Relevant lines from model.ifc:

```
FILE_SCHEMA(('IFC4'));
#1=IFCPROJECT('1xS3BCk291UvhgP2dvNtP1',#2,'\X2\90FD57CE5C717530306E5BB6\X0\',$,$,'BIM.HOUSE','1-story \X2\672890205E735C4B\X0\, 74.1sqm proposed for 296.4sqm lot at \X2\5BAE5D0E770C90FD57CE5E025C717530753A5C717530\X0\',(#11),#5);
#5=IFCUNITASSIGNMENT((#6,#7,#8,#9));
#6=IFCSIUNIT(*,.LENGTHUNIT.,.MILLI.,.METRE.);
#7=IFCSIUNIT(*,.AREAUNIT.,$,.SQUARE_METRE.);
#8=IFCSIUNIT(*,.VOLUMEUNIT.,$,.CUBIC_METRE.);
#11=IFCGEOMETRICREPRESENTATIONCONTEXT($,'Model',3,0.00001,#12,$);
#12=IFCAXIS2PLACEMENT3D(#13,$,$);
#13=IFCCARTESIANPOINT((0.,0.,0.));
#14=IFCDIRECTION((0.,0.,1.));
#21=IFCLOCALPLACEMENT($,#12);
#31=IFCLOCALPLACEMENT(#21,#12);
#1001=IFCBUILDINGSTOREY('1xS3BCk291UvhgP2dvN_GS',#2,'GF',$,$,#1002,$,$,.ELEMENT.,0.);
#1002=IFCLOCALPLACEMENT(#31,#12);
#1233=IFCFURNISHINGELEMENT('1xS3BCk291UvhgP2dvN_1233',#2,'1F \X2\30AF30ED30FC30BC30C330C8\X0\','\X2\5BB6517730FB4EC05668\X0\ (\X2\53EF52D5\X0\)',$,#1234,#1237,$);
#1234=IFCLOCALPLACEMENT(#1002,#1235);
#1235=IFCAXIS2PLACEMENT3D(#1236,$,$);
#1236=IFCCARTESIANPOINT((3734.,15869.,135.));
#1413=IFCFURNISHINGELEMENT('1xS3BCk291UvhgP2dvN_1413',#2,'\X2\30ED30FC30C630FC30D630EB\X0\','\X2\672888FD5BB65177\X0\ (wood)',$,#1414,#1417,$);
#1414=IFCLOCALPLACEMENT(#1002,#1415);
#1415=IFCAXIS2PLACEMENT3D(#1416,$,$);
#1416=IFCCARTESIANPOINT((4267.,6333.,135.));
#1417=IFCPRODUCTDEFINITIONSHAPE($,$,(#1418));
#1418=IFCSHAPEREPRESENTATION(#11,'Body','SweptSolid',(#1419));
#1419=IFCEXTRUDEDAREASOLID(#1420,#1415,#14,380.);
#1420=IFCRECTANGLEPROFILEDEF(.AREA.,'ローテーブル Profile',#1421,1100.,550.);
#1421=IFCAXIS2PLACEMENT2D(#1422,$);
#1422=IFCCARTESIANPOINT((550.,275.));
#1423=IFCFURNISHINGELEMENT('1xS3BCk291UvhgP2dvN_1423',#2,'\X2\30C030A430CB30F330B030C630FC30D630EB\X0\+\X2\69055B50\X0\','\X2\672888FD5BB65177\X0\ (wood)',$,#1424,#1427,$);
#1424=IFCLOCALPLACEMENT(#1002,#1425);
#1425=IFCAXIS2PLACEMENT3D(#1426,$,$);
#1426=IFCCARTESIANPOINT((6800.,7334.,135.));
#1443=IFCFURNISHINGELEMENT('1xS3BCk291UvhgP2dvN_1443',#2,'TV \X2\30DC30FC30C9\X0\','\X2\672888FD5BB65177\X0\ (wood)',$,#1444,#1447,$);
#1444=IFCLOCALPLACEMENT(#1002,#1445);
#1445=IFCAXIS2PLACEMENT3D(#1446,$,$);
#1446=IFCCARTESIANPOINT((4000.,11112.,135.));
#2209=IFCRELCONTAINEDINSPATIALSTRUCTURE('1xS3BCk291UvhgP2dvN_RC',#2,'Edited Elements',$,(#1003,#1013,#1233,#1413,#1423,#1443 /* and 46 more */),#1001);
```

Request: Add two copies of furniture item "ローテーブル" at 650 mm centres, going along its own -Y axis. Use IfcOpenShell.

```python
import ifcopenshell
import ifcopenshell.api.geometry
import ifcopenshell.api.root
import ifcopenshell.util.element
import ifcopenshell.util.placement

model = ifcopenshell.open("model.ifc")


def reuse_history(source, copy):
    """copy_class also copies each property set's owner history, people and application; keep the originals."""
    for rel in copy.IsDefinedBy:
        if rel.is_a("IfcRelDefinesByProperties") and (history := rel.RelatingPropertyDefinition.OwnerHistory):
            rel.RelatingPropertyDefinition.OwnerHistory = source.OwnerHistory
            ifcopenshell.util.element.remove_deep2(model, history)


source = model.by_guid("1xS3BCk291UvhgP2dvN_1413")
base = ifcopenshell.util.placement.get_local_placement(source.ObjectPlacement)
step = -base[:3, 1] * 650.0

for i in range(1, 3):
    copy = ifcopenshell.api.root.copy_class(model, product=source)
    copy.Representation = ifcopenshell.util.element.copy_deep(
        model, source.Representation, exclude=["IfcGeometricRepresentationContext", "IfcRepresentationMap"]
    )
    reuse_history(source, copy)
    matrix = base.copy()
    matrix[:3, 3] += i * step
    print("added at", matrix[:3, 3].round(3) + 0.0)
    ifcopenshell.api.geometry.edit_object_placement(model, product=copy, matrix=matrix, is_si=False)

model.write("model_v2.ifc")
```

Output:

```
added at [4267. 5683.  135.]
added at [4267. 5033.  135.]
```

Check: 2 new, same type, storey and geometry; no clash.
